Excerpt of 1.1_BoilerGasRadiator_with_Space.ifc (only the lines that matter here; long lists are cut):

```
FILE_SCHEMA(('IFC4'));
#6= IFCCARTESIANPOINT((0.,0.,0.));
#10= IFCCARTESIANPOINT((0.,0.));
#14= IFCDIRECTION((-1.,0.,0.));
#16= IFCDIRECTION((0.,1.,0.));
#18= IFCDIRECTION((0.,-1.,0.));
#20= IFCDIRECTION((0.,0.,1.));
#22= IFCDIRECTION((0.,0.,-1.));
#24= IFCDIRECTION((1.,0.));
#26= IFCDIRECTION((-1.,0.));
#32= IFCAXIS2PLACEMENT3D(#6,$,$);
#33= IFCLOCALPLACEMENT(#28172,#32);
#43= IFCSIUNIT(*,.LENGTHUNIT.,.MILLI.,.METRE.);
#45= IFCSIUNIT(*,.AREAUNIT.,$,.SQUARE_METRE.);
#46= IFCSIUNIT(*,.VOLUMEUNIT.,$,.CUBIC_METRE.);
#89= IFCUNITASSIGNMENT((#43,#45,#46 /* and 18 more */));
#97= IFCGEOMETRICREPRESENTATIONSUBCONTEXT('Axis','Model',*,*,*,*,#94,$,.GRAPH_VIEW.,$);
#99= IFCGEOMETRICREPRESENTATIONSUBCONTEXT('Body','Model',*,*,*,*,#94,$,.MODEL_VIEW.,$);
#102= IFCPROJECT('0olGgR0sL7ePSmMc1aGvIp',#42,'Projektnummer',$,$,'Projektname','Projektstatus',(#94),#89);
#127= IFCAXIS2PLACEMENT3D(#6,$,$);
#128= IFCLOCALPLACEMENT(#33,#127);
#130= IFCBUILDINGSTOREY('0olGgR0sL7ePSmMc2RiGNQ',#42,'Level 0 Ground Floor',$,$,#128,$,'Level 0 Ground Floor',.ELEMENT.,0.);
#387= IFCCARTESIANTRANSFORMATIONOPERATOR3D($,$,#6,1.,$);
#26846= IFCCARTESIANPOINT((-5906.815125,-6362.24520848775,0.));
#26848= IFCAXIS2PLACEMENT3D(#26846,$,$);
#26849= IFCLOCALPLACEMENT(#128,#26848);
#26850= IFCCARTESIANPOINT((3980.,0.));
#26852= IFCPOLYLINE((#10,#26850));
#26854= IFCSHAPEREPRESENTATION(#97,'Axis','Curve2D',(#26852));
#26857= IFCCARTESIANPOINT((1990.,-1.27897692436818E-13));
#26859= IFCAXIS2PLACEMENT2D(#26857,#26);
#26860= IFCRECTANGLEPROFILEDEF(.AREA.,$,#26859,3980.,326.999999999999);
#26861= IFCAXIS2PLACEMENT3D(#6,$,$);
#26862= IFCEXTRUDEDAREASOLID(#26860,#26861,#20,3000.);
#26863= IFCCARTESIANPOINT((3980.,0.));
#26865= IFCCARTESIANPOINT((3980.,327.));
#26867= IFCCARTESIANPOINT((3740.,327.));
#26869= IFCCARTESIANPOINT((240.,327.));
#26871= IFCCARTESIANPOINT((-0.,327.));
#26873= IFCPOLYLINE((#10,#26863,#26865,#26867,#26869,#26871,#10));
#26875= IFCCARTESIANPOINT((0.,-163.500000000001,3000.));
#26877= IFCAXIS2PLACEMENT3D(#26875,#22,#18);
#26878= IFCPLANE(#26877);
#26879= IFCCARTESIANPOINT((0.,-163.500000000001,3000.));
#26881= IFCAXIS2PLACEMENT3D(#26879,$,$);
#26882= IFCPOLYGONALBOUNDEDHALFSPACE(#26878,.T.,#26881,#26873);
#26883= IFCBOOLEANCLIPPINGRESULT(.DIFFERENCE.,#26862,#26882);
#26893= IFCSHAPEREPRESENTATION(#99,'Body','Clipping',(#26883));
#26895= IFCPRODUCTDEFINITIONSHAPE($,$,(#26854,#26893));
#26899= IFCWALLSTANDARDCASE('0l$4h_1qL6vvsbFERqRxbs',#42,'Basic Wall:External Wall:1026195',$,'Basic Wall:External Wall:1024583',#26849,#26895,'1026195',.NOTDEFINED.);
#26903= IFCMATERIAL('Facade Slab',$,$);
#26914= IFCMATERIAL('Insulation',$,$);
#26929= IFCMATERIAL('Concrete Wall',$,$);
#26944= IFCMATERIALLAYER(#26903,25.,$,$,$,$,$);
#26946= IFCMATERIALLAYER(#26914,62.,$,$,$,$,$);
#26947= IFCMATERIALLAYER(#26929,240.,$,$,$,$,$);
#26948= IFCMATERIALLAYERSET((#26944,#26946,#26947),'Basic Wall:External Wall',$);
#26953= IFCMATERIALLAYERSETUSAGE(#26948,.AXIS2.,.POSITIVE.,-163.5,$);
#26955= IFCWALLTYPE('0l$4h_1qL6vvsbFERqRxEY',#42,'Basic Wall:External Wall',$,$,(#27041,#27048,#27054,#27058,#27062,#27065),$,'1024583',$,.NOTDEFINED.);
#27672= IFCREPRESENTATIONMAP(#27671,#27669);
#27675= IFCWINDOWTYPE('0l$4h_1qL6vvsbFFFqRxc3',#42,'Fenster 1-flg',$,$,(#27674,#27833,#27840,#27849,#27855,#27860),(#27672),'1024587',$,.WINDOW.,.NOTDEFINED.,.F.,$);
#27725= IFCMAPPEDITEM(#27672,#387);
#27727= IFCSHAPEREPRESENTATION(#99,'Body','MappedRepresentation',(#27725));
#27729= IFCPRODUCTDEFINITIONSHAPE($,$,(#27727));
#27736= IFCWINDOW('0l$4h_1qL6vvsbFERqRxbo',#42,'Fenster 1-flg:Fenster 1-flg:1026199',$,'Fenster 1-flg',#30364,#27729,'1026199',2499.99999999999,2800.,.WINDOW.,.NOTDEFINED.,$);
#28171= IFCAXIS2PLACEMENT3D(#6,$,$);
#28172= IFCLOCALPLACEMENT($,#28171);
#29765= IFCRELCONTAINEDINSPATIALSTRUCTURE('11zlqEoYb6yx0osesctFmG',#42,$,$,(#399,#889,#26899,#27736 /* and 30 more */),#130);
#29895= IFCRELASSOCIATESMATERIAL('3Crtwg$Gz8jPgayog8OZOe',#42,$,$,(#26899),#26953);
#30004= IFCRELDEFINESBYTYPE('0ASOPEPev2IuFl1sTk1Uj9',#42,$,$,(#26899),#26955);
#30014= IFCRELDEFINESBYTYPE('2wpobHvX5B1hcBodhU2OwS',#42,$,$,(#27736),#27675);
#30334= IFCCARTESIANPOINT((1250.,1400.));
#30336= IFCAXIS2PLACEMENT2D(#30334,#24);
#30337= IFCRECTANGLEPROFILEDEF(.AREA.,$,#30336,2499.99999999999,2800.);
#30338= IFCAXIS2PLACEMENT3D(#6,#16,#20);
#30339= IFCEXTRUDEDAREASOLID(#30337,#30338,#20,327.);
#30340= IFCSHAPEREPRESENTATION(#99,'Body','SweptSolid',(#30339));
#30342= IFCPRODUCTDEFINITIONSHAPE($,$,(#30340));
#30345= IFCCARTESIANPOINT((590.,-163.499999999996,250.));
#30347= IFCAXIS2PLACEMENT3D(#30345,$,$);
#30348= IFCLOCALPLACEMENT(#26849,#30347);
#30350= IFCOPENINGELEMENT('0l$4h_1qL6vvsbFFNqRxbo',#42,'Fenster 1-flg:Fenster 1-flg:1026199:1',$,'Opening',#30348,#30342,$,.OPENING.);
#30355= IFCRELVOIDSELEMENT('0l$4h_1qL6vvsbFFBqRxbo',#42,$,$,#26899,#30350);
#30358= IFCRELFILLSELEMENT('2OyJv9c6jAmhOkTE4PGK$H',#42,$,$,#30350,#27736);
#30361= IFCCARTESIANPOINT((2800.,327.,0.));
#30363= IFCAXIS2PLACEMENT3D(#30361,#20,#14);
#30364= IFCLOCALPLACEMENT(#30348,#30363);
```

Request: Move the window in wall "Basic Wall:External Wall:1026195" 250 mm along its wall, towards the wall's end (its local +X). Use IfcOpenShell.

```python
import ifcopenshell
import ifcopenshell.api.geometry
import ifcopenshell.util.placement
import ifcopenshell.util.unit

model = ifcopenshell.open("1.1_BoilerGasRadiator_with_Space.ifc")
unit_scale = ifcopenshell.util.unit.calculate_unit_scale(model)

window = model.by_id(27736)
opening = window.FillsVoids[0].RelatingOpeningElement
wall = opening.VoidsElements[0].RelatingBuildingElement

wall_matrix = ifcopenshell.util.placement.get_local_placement(wall.ObjectPlacement)
shift = wall_matrix[:3, 0] * 0.25 / unit_scale
before = ifcopenshell.util.placement.get_local_placement(window.ObjectPlacement)[:3, 3].copy()

# The window is placed relative to its opening, so it follows when the opening moves.
matrix = ifcopenshell.util.placement.get_local_placement(opening.ObjectPlacement)
matrix[:3, 3] += shift
ifcopenshell.api.geometry.edit_object_placement(
    model, product=opening, matrix=matrix, is_si=False, should_transform_children=True
)

after = ifcopenshell.util.placement.get_local_placement(window.ObjectPlacement)[:3, 3]
print("window moved by", (after - before).round(3) + 0.0)

model.write("1.1_BoilerGasRadiator_with_Space_edited.ifc")
```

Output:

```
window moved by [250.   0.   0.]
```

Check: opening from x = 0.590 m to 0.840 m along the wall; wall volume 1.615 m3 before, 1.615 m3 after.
